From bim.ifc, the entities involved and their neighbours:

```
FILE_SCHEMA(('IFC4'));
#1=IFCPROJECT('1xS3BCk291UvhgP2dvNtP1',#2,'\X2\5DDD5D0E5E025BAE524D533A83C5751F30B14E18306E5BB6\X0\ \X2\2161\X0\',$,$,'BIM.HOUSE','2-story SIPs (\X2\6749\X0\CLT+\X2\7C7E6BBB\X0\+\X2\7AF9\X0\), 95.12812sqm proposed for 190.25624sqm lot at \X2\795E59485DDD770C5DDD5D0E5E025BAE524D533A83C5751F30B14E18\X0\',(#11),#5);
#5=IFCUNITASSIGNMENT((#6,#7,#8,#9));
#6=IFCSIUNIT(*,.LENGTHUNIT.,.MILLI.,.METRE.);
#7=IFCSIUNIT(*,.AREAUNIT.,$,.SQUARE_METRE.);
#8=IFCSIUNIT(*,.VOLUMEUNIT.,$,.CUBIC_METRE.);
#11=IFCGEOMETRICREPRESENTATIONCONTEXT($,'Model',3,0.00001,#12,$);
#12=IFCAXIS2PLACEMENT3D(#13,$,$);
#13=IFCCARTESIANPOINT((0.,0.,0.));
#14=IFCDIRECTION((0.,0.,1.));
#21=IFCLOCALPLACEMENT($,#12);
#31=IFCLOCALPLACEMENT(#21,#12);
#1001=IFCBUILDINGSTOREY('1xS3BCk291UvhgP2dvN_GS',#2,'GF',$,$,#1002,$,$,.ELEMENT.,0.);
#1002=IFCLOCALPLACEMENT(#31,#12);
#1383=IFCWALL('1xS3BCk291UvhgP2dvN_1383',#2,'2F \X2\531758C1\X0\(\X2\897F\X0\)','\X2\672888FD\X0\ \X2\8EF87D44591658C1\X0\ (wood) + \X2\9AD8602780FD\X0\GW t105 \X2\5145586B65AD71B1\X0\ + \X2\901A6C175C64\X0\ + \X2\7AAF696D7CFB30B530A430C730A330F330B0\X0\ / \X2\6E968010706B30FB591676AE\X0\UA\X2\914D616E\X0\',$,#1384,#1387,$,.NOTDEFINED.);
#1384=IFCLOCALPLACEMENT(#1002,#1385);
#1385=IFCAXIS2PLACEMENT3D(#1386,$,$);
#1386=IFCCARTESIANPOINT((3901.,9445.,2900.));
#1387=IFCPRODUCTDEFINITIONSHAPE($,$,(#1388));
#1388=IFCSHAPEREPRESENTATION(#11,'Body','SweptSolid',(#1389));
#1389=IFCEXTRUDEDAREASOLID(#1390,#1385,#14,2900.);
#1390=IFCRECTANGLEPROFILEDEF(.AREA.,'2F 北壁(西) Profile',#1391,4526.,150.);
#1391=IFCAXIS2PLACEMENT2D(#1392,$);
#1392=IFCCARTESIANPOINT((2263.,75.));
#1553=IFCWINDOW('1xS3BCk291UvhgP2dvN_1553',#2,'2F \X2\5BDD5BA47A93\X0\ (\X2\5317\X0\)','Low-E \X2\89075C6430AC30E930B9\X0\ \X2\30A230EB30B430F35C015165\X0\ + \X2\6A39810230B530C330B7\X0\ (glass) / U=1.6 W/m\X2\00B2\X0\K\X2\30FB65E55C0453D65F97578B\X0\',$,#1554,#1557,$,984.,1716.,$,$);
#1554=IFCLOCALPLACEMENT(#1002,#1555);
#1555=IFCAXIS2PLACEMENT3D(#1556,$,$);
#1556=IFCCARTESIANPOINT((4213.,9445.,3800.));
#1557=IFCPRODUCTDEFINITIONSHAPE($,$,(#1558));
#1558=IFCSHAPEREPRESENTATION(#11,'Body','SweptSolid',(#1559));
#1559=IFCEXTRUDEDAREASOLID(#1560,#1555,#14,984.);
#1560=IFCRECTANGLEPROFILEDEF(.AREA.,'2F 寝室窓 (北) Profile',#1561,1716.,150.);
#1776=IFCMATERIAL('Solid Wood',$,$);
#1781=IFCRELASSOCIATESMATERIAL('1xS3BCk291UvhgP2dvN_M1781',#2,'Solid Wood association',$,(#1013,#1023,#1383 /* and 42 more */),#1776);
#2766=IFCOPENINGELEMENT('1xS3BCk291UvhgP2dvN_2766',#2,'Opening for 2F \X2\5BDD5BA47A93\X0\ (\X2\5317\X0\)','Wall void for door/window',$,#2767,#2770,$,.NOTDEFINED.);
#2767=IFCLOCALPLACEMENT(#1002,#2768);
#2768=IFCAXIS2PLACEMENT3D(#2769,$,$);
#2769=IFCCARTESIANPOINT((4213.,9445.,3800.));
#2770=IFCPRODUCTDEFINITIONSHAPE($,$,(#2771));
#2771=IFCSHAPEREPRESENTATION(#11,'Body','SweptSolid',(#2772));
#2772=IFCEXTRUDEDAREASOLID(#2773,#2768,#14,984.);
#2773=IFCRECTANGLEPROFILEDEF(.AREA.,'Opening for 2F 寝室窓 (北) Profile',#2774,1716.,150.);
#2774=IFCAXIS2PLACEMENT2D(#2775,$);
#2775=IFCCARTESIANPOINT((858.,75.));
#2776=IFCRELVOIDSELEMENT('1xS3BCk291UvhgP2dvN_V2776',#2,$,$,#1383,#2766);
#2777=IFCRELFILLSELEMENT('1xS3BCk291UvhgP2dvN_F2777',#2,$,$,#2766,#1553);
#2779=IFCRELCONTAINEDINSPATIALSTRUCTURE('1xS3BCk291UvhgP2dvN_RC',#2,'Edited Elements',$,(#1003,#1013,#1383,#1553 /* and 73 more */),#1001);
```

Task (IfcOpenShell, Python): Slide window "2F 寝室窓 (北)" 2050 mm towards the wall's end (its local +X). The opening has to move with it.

```python
import ifcopenshell
import ifcopenshell.api.geometry
import ifcopenshell.util.placement

model = ifcopenshell.open("bim.ifc")

window = model.by_guid("1xS3BCk291UvhgP2dvN_1553")
opening = window.FillsVoids[0].RelatingOpeningElement
wall = opening.VoidsElements[0].RelatingBuildingElement

wall_matrix = ifcopenshell.util.placement.get_local_placement(wall.ObjectPlacement)
shift = wall_matrix[:3, 0] * 2050.0
before = ifcopenshell.util.placement.get_local_placement(window.ObjectPlacement)[:3, 3].copy()

# The window is not placed relative to its opening, so move both.
for product in (opening, window):
    matrix = ifcopenshell.util.placement.get_local_placement(product.ObjectPlacement)
    matrix[:3, 3] += shift
    ifcopenshell.api.geometry.edit_object_placement(model, product=product, matrix=matrix, is_si=False)

after = ifcopenshell.util.placement.get_local_placement(window.ObjectPlacement)[:3, 3]
print("window moved by", (after - before).round(3) + 0.0)

model.write("bim-out.ifc")
```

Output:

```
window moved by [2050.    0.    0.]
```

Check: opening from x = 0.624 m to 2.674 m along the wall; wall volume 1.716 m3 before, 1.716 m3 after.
